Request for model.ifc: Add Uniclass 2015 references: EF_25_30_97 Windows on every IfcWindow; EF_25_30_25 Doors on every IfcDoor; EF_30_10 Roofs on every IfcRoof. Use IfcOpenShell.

First a look at what the model holds.

```python
import ifcopenshell

model = ifcopenshell.open("model.ifc")
print(model.schema)
print("classifications:", [c.Name for c in model.by_type("IfcClassification")])
for ifc_class in ("IfcDoor", "IfcRoof", "IfcStair", "IfcWall", "IfcWindow"):
    print(ifc_class, len(model.by_type(ifc_class)))
```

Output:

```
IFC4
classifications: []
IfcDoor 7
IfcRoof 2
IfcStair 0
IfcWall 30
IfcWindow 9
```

```python
import ifcopenshell
import ifcopenshell.api.classification

model = ifcopenshell.open("model.ifc")

system = ifcopenshell.api.classification.add_classification(model, classification="Uniclass 2015")

codes = {
    "IfcWindow": ("EF_25_30_97", "Windows"),
    "IfcDoor": ("EF_25_30_25", "Doors"),
    "IfcRoof": ("EF_30_10", "Roofs"),
}
for ifc_class, (code, name) in codes.items():
    products = model.by_type(ifc_class)
    ifcopenshell.api.classification.add_reference(
        model, products=products, classification=system, identification=code, name=name
    )
    print(code, len(products))

model.write("model_v2.ifc")
```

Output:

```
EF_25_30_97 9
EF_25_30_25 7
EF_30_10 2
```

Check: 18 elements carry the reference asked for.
